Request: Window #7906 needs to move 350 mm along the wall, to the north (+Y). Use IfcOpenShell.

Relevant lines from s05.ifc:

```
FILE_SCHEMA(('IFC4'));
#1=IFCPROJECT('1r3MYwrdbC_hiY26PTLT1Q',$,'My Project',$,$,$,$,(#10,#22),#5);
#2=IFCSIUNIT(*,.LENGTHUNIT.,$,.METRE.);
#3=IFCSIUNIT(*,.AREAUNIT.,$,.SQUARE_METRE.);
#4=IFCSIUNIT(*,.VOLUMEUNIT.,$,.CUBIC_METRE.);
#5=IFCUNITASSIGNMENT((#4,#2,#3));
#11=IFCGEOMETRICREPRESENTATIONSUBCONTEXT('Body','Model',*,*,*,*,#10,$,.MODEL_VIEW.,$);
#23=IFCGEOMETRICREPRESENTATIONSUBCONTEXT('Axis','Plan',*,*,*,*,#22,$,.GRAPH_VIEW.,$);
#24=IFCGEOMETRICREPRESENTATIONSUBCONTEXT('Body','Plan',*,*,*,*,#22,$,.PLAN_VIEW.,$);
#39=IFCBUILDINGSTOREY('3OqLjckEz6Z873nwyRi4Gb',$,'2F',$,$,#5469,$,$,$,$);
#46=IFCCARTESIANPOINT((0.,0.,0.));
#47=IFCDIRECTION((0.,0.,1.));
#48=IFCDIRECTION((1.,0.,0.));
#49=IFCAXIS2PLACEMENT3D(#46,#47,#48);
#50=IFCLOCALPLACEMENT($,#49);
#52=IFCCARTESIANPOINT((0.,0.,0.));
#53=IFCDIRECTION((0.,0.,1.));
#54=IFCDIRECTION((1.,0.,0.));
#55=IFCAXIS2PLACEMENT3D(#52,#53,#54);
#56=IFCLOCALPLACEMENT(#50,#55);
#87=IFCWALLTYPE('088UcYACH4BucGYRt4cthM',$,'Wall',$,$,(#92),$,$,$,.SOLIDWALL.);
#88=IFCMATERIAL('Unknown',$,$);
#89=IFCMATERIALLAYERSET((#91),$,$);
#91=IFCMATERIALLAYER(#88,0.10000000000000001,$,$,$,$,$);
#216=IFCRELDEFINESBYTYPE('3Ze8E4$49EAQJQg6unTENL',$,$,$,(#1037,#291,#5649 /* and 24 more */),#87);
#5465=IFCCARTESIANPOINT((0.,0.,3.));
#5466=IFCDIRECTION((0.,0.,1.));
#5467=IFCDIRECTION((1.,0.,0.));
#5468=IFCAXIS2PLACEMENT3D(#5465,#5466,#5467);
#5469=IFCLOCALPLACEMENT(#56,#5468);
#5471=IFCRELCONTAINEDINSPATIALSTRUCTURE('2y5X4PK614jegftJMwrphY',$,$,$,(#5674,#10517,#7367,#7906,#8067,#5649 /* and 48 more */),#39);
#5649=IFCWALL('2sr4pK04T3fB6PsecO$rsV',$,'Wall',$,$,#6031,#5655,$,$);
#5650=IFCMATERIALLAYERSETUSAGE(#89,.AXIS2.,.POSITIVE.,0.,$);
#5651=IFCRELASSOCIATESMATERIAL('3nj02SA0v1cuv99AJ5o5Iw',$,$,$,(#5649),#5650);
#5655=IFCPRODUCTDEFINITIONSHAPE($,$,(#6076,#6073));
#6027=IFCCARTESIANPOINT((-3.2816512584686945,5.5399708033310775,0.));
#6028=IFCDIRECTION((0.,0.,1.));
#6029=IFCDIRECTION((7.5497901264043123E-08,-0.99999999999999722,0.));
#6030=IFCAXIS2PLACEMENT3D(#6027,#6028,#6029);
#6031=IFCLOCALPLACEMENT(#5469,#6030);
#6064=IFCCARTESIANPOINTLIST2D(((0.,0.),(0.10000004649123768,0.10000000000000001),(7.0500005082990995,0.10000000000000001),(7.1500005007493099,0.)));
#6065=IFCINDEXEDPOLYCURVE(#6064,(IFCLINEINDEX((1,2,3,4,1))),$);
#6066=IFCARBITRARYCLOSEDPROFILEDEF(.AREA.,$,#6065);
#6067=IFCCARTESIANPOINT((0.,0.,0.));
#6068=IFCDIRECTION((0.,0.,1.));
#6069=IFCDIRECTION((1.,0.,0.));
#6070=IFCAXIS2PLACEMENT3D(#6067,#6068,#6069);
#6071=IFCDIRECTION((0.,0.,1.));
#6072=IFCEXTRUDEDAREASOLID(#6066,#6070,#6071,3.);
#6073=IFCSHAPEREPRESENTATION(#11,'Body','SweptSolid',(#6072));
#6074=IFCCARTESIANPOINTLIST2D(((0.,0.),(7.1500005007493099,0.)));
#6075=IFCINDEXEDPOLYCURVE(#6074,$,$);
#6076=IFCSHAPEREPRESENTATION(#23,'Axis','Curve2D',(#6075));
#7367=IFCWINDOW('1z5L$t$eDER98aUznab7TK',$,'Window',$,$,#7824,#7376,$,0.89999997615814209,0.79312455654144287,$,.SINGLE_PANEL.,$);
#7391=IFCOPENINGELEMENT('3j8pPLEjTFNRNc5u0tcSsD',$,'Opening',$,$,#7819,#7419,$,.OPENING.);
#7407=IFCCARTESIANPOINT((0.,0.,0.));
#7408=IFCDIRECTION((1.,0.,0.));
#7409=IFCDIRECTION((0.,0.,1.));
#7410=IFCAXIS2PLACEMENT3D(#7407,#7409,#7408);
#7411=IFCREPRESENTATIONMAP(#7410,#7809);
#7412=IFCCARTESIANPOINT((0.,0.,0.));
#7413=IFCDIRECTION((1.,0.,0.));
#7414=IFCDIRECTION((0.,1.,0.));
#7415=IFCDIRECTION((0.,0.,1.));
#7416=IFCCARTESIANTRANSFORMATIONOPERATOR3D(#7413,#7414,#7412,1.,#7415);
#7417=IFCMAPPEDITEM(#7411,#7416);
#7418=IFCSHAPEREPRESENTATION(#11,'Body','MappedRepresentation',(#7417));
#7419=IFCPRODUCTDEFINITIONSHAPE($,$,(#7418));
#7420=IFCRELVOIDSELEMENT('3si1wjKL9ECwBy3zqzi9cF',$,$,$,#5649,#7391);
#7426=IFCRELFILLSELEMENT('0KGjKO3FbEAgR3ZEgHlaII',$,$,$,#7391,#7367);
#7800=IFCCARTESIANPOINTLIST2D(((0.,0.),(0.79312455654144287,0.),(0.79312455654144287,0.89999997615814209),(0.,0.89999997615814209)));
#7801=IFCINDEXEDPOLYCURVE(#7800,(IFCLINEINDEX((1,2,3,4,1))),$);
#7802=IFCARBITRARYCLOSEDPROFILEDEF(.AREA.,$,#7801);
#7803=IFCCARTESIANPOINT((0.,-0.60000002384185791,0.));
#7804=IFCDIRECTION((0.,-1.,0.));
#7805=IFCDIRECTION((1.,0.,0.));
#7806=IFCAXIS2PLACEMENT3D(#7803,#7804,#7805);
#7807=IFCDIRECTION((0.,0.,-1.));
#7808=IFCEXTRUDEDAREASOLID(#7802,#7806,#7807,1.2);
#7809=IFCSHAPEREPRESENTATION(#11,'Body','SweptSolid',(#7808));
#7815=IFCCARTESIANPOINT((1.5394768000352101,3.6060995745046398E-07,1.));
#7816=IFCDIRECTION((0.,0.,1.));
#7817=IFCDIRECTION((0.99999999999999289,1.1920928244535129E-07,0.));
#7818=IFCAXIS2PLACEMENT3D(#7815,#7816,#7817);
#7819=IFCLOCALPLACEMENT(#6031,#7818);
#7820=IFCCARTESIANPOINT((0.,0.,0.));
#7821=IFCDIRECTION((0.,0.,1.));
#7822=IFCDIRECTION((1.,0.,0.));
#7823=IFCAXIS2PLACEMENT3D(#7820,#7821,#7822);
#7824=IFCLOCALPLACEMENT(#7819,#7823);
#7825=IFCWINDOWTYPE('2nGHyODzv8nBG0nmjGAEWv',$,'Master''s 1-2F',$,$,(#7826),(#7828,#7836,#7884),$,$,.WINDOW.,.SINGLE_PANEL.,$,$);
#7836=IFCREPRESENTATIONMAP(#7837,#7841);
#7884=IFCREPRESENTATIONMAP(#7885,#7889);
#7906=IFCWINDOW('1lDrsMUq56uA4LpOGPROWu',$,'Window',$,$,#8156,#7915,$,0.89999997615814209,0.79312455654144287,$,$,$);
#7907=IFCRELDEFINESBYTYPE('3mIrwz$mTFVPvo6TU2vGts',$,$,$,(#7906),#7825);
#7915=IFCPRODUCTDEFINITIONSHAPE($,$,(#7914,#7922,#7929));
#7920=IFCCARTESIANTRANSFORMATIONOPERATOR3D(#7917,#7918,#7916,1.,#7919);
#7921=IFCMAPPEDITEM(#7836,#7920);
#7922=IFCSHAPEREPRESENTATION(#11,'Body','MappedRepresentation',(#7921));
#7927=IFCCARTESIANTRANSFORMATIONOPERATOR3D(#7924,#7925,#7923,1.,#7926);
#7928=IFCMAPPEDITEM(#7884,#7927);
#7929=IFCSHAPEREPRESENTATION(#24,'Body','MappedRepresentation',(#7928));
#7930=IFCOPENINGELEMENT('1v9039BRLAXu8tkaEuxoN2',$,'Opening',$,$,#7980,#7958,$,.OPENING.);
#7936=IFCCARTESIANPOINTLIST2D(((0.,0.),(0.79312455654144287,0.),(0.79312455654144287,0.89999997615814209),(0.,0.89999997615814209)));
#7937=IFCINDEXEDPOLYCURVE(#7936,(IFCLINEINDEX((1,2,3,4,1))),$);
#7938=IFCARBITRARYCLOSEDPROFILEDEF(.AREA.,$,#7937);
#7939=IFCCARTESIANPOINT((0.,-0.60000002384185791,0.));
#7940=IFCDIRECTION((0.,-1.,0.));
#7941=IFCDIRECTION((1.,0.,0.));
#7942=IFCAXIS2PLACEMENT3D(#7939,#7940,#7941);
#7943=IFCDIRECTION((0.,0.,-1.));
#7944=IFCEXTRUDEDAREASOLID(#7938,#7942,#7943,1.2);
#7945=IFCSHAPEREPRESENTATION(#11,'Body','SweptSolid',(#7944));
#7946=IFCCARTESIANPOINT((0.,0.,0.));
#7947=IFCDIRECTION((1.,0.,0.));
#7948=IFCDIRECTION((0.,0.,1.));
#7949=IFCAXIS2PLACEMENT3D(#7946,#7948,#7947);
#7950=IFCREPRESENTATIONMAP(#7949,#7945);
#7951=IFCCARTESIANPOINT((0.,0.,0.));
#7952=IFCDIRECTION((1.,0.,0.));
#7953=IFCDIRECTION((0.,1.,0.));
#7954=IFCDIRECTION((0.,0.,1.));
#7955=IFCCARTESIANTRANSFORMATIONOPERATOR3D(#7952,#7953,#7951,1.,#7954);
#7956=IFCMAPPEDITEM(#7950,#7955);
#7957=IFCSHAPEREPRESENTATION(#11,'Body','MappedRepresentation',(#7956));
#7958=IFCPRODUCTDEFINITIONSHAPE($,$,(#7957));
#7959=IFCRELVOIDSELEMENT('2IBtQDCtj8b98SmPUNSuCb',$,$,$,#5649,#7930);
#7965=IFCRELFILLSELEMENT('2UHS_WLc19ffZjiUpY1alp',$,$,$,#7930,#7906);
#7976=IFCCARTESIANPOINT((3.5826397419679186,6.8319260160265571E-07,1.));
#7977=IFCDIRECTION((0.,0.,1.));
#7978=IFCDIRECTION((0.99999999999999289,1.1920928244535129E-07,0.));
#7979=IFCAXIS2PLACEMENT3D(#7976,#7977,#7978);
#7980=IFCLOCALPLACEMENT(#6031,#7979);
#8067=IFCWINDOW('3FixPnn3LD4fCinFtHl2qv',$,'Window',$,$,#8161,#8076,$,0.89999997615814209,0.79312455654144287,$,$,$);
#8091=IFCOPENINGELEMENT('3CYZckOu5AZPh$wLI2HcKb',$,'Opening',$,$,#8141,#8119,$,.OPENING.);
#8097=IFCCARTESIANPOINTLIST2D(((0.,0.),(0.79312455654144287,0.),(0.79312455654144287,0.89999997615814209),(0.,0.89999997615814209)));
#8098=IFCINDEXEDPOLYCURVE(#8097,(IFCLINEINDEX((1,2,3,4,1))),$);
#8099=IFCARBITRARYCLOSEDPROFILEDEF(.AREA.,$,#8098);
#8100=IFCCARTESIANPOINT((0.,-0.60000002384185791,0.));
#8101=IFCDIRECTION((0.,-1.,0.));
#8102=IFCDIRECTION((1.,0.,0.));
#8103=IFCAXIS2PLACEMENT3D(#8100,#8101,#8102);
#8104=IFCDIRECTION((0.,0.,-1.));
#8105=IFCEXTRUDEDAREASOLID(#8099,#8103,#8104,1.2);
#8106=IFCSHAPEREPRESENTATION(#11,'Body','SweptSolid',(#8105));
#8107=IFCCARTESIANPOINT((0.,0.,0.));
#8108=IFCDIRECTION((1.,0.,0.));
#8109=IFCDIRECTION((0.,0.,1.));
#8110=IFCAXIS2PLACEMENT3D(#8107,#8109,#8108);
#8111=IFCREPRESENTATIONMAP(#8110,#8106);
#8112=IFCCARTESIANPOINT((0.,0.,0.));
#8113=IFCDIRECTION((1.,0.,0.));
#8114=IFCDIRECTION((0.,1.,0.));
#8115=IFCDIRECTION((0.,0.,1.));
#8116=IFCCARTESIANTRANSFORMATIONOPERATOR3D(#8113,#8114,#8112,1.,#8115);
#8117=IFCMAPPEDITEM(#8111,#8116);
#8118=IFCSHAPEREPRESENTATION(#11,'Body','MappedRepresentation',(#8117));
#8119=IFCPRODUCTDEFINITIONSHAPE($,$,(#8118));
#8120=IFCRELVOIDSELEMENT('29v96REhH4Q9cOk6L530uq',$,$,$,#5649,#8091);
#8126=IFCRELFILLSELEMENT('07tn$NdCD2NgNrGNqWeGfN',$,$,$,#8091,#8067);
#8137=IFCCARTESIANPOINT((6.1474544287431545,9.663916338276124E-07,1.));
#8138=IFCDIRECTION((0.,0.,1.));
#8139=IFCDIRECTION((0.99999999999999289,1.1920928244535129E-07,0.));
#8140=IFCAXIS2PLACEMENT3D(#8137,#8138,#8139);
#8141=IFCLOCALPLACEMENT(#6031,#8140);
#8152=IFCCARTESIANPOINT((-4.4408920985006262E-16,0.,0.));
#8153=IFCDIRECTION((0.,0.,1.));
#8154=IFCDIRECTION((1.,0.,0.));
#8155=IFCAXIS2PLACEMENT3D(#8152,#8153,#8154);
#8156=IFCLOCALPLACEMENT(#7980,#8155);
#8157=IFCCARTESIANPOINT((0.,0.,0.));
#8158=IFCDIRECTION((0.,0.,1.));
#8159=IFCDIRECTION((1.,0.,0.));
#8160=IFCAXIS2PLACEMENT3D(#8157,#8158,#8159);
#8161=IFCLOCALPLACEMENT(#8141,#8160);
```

```python
import ifcopenshell
import ifcopenshell.api.geometry
import ifcopenshell.util.placement
import ifcopenshell.util.unit

model = ifcopenshell.open("s05.ifc")
unit_scale = ifcopenshell.util.unit.calculate_unit_scale(model)

window = model.by_guid("1lDrsMUq56uA4LpOGPROWu")
opening = window.FillsVoids[0].RelatingOpeningElement
wall = opening.VoidsElements[0].RelatingBuildingElement

wall_matrix = ifcopenshell.util.placement.get_local_placement(wall.ObjectPlacement)
shift = wall_matrix[:3, 0] * -0.35 / unit_scale
before = ifcopenshell.util.placement.get_local_placement(window.ObjectPlacement)[:3, 3].copy()

# The window is placed relative to its opening, so it follows when the opening moves.
matrix = ifcopenshell.util.placement.get_local_placement(opening.ObjectPlacement)
matrix[:3, 3] += shift
ifcopenshell.api.geometry.edit_object_placement(
    model, product=opening, matrix=matrix, is_si=False, should_transform_children=True
)

after = ifcopenshell.util.placement.get_local_placement(window.ObjectPlacement)[:3, 3]
print("window moved by", (after - before).round(3) + 0.0)

model.write("s05_rev.ifc")
```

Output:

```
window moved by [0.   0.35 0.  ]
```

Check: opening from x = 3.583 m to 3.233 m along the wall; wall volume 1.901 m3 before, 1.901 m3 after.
